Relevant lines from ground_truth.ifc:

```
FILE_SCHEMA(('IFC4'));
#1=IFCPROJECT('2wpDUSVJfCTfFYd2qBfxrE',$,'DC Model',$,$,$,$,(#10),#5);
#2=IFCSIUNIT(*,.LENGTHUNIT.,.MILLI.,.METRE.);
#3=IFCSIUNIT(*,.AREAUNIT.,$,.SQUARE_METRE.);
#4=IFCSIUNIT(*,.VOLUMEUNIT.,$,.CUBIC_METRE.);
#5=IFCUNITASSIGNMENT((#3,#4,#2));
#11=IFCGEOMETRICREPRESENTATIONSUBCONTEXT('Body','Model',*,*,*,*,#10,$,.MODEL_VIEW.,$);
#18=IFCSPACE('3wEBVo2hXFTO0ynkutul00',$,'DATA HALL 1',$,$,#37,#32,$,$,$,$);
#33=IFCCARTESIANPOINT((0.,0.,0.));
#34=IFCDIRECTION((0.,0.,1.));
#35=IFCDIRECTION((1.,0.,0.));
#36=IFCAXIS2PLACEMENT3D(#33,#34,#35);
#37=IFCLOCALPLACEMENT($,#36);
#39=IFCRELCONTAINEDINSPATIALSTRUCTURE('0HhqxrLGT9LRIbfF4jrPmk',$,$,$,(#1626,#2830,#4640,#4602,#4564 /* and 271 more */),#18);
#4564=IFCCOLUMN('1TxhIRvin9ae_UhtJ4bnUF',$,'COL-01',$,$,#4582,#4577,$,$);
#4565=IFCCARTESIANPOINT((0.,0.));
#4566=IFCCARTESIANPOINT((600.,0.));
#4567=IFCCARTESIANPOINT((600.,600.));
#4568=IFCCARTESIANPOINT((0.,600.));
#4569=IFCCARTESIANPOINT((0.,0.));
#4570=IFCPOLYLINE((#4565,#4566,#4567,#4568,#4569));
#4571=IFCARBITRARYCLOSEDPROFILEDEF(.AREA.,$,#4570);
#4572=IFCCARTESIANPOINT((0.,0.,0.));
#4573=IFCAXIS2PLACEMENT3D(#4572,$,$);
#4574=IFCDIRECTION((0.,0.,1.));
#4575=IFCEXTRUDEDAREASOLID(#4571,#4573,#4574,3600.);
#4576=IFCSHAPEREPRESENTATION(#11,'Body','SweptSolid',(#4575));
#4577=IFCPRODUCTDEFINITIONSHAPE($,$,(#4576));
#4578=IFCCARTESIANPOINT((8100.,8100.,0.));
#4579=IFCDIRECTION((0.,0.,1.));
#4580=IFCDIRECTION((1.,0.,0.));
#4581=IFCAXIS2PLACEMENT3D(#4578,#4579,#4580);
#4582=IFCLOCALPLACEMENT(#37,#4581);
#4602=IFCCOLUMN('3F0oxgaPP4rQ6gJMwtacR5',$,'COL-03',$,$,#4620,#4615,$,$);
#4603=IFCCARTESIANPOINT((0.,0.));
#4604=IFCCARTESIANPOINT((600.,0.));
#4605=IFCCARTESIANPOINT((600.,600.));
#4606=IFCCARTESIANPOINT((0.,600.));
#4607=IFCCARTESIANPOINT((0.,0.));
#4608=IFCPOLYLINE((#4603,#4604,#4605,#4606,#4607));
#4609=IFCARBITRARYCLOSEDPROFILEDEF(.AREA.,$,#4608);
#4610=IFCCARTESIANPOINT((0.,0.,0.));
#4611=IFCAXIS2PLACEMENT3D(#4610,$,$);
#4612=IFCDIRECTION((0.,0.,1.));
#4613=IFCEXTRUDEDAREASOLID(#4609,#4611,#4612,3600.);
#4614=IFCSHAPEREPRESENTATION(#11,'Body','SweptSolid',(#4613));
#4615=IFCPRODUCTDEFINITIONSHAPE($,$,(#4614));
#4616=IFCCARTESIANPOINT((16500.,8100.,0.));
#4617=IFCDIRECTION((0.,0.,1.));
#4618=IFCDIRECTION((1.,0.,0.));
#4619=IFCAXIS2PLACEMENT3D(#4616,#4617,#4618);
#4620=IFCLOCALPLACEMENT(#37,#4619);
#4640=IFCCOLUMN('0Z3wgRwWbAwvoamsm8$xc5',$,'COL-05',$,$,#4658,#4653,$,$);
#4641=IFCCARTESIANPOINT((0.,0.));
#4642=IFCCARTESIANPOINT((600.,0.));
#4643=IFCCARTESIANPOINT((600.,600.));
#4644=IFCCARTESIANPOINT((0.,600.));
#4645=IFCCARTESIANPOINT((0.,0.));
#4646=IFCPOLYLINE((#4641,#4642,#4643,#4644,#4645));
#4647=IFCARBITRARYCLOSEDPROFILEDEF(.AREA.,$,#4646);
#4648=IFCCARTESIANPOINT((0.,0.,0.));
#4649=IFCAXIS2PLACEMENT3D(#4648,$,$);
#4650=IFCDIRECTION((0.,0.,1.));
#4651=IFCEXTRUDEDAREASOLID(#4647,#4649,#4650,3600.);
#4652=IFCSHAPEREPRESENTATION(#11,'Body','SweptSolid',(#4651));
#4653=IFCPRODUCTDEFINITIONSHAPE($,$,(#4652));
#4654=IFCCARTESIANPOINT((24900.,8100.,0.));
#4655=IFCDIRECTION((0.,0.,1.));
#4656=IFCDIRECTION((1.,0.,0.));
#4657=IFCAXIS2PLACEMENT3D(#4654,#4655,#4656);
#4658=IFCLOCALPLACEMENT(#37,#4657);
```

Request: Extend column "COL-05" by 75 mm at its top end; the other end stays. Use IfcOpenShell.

```python
import ifcopenshell
import ifcopenshell.util.representation

model = ifcopenshell.open("ground_truth.ifc")

member = model.by_id(4640)
change = 75.0

# The extrusion runs towards the end named, so only its depth changes.
body = ifcopenshell.util.representation.get_representation(member, "Model", "Body")
solid = body.Items[0]
old_length = solid.Depth
solid.Depth += change

print(f"length {old_length:g} -> {solid.Depth:g}")

model.write("ground_truth_updated.ifc")
```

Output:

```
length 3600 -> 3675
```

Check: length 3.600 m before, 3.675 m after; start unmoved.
